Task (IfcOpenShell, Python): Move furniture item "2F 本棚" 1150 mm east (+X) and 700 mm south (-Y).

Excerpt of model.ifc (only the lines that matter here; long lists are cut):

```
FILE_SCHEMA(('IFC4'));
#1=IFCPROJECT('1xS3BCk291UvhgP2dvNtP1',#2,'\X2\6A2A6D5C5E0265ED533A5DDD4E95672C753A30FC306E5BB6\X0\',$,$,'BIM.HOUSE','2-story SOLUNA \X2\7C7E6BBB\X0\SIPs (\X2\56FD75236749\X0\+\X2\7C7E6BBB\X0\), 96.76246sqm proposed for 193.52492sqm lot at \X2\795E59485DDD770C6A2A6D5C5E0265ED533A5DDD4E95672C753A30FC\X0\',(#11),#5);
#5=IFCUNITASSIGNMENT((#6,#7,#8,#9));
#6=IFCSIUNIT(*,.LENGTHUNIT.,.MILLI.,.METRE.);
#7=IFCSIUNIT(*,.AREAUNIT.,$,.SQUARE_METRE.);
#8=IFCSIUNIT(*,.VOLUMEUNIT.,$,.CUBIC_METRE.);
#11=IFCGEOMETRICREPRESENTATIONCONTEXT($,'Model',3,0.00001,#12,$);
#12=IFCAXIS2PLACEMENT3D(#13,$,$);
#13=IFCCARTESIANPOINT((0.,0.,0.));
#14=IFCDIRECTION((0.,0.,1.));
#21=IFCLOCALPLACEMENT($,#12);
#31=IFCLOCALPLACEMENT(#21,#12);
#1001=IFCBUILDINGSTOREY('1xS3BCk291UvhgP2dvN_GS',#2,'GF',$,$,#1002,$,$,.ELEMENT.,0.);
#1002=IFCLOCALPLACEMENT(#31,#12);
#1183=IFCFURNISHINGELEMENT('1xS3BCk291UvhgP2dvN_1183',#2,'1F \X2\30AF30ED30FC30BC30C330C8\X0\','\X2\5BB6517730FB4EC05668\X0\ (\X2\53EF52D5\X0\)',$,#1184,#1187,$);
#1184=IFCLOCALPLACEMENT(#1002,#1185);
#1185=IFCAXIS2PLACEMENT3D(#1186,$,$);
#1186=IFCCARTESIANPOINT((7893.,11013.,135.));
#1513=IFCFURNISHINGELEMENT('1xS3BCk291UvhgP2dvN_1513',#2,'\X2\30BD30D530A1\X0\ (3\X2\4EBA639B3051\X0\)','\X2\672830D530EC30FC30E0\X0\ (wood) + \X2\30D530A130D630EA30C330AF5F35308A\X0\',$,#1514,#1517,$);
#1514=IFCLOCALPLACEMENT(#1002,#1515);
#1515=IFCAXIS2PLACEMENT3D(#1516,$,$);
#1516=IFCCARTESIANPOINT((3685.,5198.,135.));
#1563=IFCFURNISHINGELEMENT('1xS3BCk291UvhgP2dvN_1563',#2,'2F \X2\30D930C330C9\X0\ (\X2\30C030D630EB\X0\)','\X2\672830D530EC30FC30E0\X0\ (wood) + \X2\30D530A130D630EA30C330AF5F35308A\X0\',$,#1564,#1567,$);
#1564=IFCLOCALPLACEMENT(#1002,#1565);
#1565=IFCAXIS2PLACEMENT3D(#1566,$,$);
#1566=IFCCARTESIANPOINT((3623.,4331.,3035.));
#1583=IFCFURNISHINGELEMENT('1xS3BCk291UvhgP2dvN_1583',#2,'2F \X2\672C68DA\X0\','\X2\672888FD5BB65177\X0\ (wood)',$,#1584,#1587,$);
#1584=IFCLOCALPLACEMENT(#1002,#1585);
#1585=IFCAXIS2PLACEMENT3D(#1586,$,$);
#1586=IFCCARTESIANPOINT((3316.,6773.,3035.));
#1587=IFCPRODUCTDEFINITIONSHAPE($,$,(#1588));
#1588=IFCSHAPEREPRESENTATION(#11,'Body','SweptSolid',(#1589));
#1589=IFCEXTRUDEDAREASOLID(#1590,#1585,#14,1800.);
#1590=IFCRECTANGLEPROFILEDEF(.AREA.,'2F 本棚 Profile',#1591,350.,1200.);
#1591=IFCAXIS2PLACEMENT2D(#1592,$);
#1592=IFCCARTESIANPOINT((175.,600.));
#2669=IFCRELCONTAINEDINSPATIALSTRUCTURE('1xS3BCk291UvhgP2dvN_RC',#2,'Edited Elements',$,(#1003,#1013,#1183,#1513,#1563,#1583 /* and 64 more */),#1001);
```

```python
import ifcopenshell
import ifcopenshell.api.geometry
import ifcopenshell.util.placement

model = ifcopenshell.open("model.ifc")

item = model.by_guid("1xS3BCk291UvhgP2dvN_1583")
matrix = ifcopenshell.util.placement.get_local_placement(item.ObjectPlacement)
matrix[0, 3] += 1150.0
matrix[1, 3] -= 700.0
ifcopenshell.api.geometry.edit_object_placement(model, product=item, matrix=matrix, is_si=False)

print(ifcopenshell.util.placement.get_local_placement(item.ObjectPlacement).round(3) + 0.0)

model.write("model_updated.ifc")
```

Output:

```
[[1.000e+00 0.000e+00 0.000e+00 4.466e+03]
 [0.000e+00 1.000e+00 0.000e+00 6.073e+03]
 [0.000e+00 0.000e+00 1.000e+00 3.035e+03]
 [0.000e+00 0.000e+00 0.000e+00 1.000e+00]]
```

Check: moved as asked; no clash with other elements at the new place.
